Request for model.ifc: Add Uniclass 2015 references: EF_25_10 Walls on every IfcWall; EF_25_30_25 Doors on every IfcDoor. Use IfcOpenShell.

First a look at what the model holds.

```python
import ifcopenshell

model = ifcopenshell.open("model.ifc")
print(model.schema)
print("classifications:", [c.Name for c in model.by_type("IfcClassification")])
for ifc_class in ("IfcDoor", "IfcRoof", "IfcStair", "IfcWall", "IfcWindow"):
    print(ifc_class, len(model.by_type(ifc_class)))
```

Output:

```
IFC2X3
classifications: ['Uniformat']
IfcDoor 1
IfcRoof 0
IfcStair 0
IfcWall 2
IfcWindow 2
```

```python
import ifcopenshell
import ifcopenshell.api.classification

model = ifcopenshell.open("model.ifc")

# IFC2X3 requires Source and Edition and has no link from the project to the system.
system = model.create_entity("IfcClassification", Source="NBS", Edition="2015", Name="Uniclass 2015")

codes = {
    "IfcWall": ("EF_25_10", "Walls"),
    "IfcDoor": ("EF_25_30_25", "Doors"),
}
for ifc_class, (code, name) in codes.items():
    products = model.by_type(ifc_class)
    ifcopenshell.api.classification.add_reference(
        model, products=products, classification=system, identification=code, name=name
    )
    print(code, len(products))

model.write("model_updated.ifc")
```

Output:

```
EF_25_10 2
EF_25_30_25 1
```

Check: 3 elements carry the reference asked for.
